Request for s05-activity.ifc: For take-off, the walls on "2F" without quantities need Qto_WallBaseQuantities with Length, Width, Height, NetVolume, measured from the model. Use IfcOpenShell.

First a look at what the model holds.

```python
import ifcopenshell
import ifcopenshell.util.element
import ifcopenshell.util.unit

model = ifcopenshell.open("s05-activity.ifc")
print(model.schema)
for unit_type in ("LENGTHUNIT", "AREAUNIT", "VOLUMEUNIT"):
    print(unit_type, ifcopenshell.util.unit.calculate_unit_scale(model, unit_type))
storey = next(s for s in model.by_type("IfcBuildingStorey") if s.Name == "2F")
walls = [e for e in ifcopenshell.util.element.get_decomposition(storey) if e.is_a("IfcWall")]
for e in sorted(walls, key=lambda e: e.id()):
    print(e.id(), e.is_a(), e.Name, list(ifcopenshell.util.element.get_psets(e, qtos_only=True)), sep=" | ")
```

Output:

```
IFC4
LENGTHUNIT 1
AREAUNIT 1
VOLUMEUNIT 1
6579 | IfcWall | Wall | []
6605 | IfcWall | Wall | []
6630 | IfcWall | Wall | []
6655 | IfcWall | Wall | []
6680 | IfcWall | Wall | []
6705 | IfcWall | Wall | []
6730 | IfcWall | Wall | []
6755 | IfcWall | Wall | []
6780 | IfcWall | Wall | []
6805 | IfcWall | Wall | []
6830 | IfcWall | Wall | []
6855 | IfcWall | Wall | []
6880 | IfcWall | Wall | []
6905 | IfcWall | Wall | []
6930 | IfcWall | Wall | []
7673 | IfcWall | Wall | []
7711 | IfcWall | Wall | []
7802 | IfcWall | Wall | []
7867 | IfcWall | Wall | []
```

```python
import ifcopenshell
import ifcopenshell.api.pset
import ifcopenshell.geom
import ifcopenshell.util.element
import ifcopenshell.util.shape
import ifcopenshell.util.unit

model = ifcopenshell.open("s05-activity.ifc")
unit_scale = ifcopenshell.util.unit.calculate_unit_scale(model)
volume_scale = ifcopenshell.util.unit.calculate_unit_scale(model, "VOLUMEUNIT")
settings = ifcopenshell.geom.settings()

storey = next(s for s in model.by_type("IfcBuildingStorey") if s.Name == "2F")
walls = [e for e in ifcopenshell.util.element.get_decomposition(storey) if e.is_a("IfcWall")]

for e in sorted(walls, key=lambda e: e.id()):
    if ifcopenshell.util.element.get_psets(e, qtos_only=True, should_inherit=False):
        continue
    # Geometry comes back in metres, in the element's own axes.
    shape = ifcopenshell.geom.create_shape(settings, e)
    values = {
        "Length": ifcopenshell.util.shape.get_x(shape.geometry) / unit_scale,
        "Width": ifcopenshell.util.shape.get_y(shape.geometry) / unit_scale,
        "Height": ifcopenshell.util.shape.get_z(shape.geometry) / unit_scale,
        "NetVolume": ifcopenshell.util.shape.get_volume(shape.geometry) / volume_scale,
    }
    qto = ifcopenshell.api.pset.add_qto(model, product=e, name="Qto_WallBaseQuantities")
    ifcopenshell.api.pset.edit_qto(model, qto=qto, properties=values)
    print(e.id(), {k: round(v, 3) for k, v in values.items()})

model.write("s05-activity_v2.ifc")
```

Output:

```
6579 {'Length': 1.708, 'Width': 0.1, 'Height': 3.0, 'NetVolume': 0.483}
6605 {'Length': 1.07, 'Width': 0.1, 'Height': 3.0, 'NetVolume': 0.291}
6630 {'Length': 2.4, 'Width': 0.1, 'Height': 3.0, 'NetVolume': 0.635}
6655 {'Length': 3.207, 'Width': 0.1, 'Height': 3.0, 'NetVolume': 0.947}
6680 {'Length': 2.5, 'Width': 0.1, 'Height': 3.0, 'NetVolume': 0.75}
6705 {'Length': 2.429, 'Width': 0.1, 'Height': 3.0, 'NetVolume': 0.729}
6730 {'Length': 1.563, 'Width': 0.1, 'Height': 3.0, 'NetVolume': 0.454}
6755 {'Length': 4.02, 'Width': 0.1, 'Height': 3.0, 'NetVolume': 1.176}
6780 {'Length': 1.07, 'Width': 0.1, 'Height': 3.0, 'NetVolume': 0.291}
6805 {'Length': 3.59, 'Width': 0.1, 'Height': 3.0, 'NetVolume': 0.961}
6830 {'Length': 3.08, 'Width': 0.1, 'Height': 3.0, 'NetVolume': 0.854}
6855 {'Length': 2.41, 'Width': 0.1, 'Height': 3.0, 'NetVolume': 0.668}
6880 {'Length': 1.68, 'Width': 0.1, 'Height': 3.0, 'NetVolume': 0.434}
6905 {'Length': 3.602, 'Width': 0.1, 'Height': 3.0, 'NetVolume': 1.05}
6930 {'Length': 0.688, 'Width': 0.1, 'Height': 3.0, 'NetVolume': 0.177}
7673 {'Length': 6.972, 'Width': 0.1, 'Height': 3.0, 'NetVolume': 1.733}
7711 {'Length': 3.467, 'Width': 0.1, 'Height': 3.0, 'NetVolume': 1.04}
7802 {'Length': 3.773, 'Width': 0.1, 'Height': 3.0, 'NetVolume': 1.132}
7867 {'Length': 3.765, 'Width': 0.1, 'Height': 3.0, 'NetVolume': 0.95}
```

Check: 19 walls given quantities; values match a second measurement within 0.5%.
